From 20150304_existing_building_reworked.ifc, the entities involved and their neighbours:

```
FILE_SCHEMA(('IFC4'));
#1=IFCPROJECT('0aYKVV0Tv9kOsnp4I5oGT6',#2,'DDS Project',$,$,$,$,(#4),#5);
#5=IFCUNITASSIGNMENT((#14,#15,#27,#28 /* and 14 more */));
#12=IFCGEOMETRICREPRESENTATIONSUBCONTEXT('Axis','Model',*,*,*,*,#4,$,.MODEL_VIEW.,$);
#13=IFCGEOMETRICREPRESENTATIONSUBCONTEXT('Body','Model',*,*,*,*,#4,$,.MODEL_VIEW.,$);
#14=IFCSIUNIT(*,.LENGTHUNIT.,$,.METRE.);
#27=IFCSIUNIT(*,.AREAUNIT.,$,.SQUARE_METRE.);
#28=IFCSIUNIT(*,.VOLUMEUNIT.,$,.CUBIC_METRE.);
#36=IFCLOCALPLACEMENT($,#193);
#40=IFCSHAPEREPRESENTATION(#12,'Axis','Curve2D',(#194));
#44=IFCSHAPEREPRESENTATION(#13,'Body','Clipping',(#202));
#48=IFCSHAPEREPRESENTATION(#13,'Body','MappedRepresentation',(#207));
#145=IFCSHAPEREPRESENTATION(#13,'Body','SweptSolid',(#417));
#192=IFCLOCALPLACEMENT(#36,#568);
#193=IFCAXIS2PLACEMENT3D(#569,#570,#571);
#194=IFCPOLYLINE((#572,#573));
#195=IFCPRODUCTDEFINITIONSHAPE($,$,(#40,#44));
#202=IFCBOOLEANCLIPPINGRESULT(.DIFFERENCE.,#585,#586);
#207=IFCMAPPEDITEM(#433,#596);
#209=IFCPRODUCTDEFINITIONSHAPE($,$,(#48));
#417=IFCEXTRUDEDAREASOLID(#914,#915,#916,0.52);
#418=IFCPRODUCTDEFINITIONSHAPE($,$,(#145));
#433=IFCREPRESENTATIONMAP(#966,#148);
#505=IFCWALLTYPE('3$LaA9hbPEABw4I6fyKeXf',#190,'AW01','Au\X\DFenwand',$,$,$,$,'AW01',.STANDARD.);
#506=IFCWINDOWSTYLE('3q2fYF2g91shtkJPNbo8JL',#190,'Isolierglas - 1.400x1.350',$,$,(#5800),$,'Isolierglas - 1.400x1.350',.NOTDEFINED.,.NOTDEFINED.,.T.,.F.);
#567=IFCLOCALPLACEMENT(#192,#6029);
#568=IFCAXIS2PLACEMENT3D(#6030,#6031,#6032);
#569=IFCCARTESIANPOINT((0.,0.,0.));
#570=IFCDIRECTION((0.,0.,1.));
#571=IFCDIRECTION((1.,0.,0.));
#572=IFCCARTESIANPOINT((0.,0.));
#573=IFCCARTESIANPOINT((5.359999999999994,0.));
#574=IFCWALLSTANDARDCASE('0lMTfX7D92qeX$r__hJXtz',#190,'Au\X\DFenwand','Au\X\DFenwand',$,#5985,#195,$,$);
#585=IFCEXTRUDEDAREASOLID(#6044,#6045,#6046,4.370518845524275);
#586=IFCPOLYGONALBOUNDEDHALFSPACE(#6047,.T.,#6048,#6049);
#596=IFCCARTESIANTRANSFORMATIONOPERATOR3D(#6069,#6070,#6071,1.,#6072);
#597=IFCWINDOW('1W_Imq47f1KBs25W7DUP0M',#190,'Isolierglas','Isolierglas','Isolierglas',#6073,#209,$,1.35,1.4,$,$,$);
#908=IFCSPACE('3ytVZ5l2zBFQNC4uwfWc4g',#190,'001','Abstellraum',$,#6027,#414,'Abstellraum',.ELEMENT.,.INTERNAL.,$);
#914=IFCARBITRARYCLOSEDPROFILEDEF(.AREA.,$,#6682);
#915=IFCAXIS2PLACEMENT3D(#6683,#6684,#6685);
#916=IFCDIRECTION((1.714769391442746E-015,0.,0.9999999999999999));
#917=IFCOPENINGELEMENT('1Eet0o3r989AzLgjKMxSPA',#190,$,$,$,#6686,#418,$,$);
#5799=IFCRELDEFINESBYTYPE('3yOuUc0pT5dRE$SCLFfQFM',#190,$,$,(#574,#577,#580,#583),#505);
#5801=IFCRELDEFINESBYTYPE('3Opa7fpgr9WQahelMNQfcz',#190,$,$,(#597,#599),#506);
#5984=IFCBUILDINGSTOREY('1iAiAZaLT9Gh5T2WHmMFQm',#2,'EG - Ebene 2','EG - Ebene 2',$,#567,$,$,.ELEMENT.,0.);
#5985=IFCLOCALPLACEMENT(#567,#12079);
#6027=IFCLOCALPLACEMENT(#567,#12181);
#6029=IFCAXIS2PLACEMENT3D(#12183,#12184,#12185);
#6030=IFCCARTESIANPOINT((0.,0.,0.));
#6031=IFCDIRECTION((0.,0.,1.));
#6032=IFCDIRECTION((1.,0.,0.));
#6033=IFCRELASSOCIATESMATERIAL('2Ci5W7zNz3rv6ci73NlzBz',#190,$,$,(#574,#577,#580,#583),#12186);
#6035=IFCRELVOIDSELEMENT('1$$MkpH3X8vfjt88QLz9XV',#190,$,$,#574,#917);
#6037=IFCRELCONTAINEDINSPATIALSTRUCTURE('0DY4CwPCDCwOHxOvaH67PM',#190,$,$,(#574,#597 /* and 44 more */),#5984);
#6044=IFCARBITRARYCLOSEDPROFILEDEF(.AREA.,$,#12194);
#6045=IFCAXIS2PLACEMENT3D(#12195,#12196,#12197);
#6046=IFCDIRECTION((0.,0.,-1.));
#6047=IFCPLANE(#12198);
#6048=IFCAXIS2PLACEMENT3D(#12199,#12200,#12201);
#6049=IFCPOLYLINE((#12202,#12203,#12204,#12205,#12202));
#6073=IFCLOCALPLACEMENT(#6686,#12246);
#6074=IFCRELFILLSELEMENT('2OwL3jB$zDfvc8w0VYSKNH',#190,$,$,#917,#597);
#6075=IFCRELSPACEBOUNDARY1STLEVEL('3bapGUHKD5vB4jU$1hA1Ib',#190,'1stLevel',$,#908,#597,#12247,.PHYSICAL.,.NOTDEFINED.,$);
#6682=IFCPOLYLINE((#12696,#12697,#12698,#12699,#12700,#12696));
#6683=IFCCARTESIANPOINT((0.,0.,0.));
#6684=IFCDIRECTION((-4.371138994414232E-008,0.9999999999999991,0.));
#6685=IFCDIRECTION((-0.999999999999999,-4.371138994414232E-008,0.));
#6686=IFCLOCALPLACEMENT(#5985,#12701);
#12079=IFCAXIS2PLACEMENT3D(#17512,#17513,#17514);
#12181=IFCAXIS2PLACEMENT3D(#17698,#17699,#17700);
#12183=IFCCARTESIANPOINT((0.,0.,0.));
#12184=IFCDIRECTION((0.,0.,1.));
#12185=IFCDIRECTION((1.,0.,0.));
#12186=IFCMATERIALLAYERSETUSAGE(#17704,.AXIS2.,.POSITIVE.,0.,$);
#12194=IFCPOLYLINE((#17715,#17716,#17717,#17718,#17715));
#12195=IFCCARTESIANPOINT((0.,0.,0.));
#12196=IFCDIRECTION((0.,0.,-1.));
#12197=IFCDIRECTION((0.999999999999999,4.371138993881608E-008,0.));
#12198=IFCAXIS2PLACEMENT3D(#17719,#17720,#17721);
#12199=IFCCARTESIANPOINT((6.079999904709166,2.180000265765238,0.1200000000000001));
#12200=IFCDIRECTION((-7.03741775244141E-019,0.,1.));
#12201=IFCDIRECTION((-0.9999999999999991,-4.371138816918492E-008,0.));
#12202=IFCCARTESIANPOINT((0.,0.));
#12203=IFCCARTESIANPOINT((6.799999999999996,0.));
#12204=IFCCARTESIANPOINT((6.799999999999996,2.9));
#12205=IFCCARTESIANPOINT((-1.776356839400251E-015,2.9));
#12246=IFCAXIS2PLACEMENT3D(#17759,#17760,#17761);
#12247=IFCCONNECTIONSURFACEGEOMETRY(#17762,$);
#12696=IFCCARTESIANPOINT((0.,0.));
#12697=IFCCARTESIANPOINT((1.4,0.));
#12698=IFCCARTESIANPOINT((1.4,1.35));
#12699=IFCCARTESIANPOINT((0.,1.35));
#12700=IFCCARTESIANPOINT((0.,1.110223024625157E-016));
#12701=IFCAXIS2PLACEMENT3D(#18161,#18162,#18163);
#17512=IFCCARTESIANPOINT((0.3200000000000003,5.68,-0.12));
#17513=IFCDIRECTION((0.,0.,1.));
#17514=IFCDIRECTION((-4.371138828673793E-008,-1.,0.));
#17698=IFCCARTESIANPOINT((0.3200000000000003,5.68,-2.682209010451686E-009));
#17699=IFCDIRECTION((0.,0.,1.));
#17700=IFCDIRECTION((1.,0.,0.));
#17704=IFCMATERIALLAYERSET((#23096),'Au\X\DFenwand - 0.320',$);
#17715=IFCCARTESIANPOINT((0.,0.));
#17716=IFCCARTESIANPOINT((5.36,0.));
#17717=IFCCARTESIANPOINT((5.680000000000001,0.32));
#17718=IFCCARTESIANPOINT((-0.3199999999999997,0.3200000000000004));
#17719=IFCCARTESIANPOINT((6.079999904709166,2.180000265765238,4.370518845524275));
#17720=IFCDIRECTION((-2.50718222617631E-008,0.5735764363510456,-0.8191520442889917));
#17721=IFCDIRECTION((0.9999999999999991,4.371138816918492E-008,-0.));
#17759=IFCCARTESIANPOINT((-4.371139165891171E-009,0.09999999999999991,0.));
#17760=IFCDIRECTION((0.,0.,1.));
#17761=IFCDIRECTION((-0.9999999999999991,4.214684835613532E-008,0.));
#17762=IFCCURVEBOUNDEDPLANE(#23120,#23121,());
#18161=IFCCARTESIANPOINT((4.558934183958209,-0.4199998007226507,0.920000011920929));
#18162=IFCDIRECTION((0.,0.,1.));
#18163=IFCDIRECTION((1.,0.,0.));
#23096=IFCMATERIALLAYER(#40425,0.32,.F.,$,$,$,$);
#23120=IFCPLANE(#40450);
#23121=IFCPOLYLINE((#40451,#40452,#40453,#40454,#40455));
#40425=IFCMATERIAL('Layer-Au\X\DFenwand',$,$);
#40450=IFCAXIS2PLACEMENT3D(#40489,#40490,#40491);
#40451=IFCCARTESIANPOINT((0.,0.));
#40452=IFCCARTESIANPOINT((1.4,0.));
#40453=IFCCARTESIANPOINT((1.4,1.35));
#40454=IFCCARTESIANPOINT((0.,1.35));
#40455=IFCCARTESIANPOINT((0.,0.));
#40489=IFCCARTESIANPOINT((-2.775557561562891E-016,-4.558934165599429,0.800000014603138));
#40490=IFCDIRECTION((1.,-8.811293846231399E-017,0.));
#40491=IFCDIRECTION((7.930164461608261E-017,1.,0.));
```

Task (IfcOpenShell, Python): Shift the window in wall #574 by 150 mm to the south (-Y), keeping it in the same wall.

```python
import numpy as np
import ifcopenshell
import ifcopenshell.api.geometry
import ifcopenshell.util.placement

model = ifcopenshell.open("20150304_existing_building_reworked.ifc")

window = model.by_id(597)
opening = window.FillsVoids[0].RelatingOpeningElement
wall = opening.VoidsElements[0].RelatingBuildingElement

wall_matrix = ifcopenshell.util.placement.get_local_placement(wall.ObjectPlacement)
shift = wall_matrix[:3, 0] * 0.15
before = ifcopenshell.util.placement.get_local_placement(window.ObjectPlacement)[:3, 3].copy()

# The window is placed relative to its opening, so it follows when the opening moves.
matrix = ifcopenshell.util.placement.get_local_placement(opening.ObjectPlacement)
matrix[:3, 3] += shift
ifcopenshell.api.geometry.edit_object_placement(
    model, product=opening, matrix=matrix, is_si=False, should_transform_children=True
)

# Space boundary surfaces are stored in each space's coordinates; move them too.
for rel in window.ProvidesBoundaries:
    if not rel.ConnectionGeometry:
        continue
    surface = rel.ConnectionGeometry.SurfaceOnRelatingElement.BasisSurface
    space_matrix = ifcopenshell.util.placement.get_local_placement(rel.RelatingSpace.ObjectPlacement)
    point = np.array(surface.Position.Location.Coordinates) + space_matrix[:3, :3].T @ shift
    surface.Position = model.createIfcAxis2Placement3D(
        model.createIfcCartesianPoint(point.tolist()), surface.Position.Axis, surface.Position.RefDirection
    )

after = ifcopenshell.util.placement.get_local_placement(window.ObjectPlacement)[:3, 3]
print("window moved by", (after - before).round(3) + 0.0)

model.write("20150304_existing_building_reworked_edited.ifc")
```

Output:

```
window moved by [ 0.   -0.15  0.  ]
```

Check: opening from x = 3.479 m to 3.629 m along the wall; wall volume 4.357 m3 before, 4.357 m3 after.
